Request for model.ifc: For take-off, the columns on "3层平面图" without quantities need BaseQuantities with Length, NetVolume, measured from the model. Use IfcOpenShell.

First a look at what the model holds.

```python
import ifcopenshell
import ifcopenshell.util.element
import ifcopenshell.util.unit

model = ifcopenshell.open("model.ifc")
print(model.schema)
for unit_type in ("LENGTHUNIT", "AREAUNIT", "VOLUMEUNIT"):
    print(unit_type, ifcopenshell.util.unit.calculate_unit_scale(model, unit_type))
storey = next(s for s in model.by_type("IfcBuildingStorey") if s.Name == "3层平面图")
columns = [e for e in ifcopenshell.util.element.get_decomposition(storey) if e.is_a("IfcColumn")]
for e in sorted(columns, key=lambda e: e.id()):
    print(e.id(), e.is_a(), e.Name, list(ifcopenshell.util.element.get_psets(e, qtos_only=True)), sep=" | ")
```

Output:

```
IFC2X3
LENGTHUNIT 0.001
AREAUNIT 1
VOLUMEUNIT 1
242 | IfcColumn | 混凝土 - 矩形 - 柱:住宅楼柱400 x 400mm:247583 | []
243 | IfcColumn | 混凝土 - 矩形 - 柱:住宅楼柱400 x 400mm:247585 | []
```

```python
import ifcopenshell
import ifcopenshell.api.pset
import ifcopenshell.geom
import ifcopenshell.util.element
import ifcopenshell.util.shape
import ifcopenshell.util.unit

model = ifcopenshell.open("model.ifc")
unit_scale = ifcopenshell.util.unit.calculate_unit_scale(model)
volume_scale = ifcopenshell.util.unit.calculate_unit_scale(model, "VOLUMEUNIT")
settings = ifcopenshell.geom.settings()

storey = next(s for s in model.by_type("IfcBuildingStorey") if s.Name == "3层平面图")
columns = [e for e in ifcopenshell.util.element.get_decomposition(storey) if e.is_a("IfcColumn")]

for e in sorted(columns, key=lambda e: e.id()):
    if ifcopenshell.util.element.get_psets(e, qtos_only=True, should_inherit=False):
        continue
    # Geometry comes back in metres, in the element's own axes.
    shape = ifcopenshell.geom.create_shape(settings, e)
    values = {
        "Length": ifcopenshell.util.shape.get_z(shape.geometry) / unit_scale,
        "NetVolume": ifcopenshell.util.shape.get_volume(shape.geometry) / volume_scale,
    }
    qto = ifcopenshell.api.pset.add_qto(model, product=e, name="BaseQuantities")
    ifcopenshell.api.pset.edit_qto(model, qto=qto, properties=values)
    print(e.id(), {k: round(v, 3) for k, v in values.items()})

model.write("model_rev.ifc")
```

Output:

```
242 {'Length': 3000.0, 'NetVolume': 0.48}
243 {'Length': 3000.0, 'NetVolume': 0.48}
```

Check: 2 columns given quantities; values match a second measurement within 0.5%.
